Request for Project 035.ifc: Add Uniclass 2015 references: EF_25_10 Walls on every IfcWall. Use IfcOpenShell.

First a look at what the model holds.

```python
import ifcopenshell

model = ifcopenshell.open("Project 035.ifc")
print(model.schema)
print("classifications:", [c.Name for c in model.by_type("IfcClassification")])
for ifc_class in ("IfcDoor", "IfcRoof", "IfcStair", "IfcWall", "IfcWindow"):
    print(ifc_class, len(model.by_type(ifc_class)))
```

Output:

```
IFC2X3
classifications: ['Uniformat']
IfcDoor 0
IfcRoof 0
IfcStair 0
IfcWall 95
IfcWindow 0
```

```python
import ifcopenshell
import ifcopenshell.api.classification

model = ifcopenshell.open("Project 035.ifc")

# IFC2X3 requires Source and Edition and has no link from the project to the system.
system = model.create_entity("IfcClassification", Source="NBS", Edition="2015", Name="Uniclass 2015")

codes = {
    "IfcWall": ("EF_25_10", "Walls"),
}
for ifc_class, (code, name) in codes.items():
    products = model.by_type(ifc_class)
    ifcopenshell.api.classification.add_reference(
        model, products=products, classification=system, identification=code, name=name
    )
    print(code, len(products))

model.write("Project 035_edited.ifc")
```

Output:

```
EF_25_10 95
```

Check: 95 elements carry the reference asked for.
